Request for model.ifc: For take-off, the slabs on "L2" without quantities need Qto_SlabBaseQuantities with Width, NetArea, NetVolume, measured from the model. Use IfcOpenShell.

First a look at what the model holds.

```python
import ifcopenshell
import ifcopenshell.util.element
import ifcopenshell.util.unit

model = ifcopenshell.open("model.ifc")
print(model.schema)
for unit_type in ("LENGTHUNIT", "AREAUNIT", "VOLUMEUNIT"):
    print(unit_type, ifcopenshell.util.unit.calculate_unit_scale(model, unit_type))
storey = next(s for s in model.by_type("IfcBuildingStorey") if s.Name == "L2")
slabs = [e for e in ifcopenshell.util.element.get_decomposition(storey) if e.is_a("IfcSlab")]
for e in sorted(slabs, key=lambda e: e.id()):
    print(e.id(), e.is_a(), e.Name, list(ifcopenshell.util.element.get_psets(e, qtos_only=True)), sep=" | ")
```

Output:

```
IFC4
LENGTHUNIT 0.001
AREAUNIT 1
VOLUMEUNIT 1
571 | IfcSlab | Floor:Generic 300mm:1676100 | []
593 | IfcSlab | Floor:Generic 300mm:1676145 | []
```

```python
import ifcopenshell
import ifcopenshell.api.pset
import ifcopenshell.geom
import ifcopenshell.util.element
import ifcopenshell.util.shape
import ifcopenshell.util.unit

model = ifcopenshell.open("model.ifc")
unit_scale = ifcopenshell.util.unit.calculate_unit_scale(model)
area_scale = ifcopenshell.util.unit.calculate_unit_scale(model, "AREAUNIT")
volume_scale = ifcopenshell.util.unit.calculate_unit_scale(model, "VOLUMEUNIT")
settings = ifcopenshell.geom.settings()

storey = next(s for s in model.by_type("IfcBuildingStorey") if s.Name == "L2")
slabs = [e for e in ifcopenshell.util.element.get_decomposition(storey) if e.is_a("IfcSlab")]

for e in sorted(slabs, key=lambda e: e.id()):
    if ifcopenshell.util.element.get_psets(e, qtos_only=True, should_inherit=False):
        continue
    # Geometry comes back in metres, in the element's own axes.
    shape = ifcopenshell.geom.create_shape(settings, e)
    values = {
        "Width": ifcopenshell.util.shape.get_z(shape.geometry) / unit_scale,
        "NetArea": ifcopenshell.util.shape.get_footprint_area(shape.geometry) / area_scale,
        "NetVolume": ifcopenshell.util.shape.get_volume(shape.geometry) / volume_scale,
    }
    qto = ifcopenshell.api.pset.add_qto(model, product=e, name="Qto_SlabBaseQuantities")
    ifcopenshell.api.pset.edit_qto(model, qto=qto, properties=values)
    print(e.id(), {k: round(v, 3) for k, v in values.items()})

model.write("model_updated.ifc")
```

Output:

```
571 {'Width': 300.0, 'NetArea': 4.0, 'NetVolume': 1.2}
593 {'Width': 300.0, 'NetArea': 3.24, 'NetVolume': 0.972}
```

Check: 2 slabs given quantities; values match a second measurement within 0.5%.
